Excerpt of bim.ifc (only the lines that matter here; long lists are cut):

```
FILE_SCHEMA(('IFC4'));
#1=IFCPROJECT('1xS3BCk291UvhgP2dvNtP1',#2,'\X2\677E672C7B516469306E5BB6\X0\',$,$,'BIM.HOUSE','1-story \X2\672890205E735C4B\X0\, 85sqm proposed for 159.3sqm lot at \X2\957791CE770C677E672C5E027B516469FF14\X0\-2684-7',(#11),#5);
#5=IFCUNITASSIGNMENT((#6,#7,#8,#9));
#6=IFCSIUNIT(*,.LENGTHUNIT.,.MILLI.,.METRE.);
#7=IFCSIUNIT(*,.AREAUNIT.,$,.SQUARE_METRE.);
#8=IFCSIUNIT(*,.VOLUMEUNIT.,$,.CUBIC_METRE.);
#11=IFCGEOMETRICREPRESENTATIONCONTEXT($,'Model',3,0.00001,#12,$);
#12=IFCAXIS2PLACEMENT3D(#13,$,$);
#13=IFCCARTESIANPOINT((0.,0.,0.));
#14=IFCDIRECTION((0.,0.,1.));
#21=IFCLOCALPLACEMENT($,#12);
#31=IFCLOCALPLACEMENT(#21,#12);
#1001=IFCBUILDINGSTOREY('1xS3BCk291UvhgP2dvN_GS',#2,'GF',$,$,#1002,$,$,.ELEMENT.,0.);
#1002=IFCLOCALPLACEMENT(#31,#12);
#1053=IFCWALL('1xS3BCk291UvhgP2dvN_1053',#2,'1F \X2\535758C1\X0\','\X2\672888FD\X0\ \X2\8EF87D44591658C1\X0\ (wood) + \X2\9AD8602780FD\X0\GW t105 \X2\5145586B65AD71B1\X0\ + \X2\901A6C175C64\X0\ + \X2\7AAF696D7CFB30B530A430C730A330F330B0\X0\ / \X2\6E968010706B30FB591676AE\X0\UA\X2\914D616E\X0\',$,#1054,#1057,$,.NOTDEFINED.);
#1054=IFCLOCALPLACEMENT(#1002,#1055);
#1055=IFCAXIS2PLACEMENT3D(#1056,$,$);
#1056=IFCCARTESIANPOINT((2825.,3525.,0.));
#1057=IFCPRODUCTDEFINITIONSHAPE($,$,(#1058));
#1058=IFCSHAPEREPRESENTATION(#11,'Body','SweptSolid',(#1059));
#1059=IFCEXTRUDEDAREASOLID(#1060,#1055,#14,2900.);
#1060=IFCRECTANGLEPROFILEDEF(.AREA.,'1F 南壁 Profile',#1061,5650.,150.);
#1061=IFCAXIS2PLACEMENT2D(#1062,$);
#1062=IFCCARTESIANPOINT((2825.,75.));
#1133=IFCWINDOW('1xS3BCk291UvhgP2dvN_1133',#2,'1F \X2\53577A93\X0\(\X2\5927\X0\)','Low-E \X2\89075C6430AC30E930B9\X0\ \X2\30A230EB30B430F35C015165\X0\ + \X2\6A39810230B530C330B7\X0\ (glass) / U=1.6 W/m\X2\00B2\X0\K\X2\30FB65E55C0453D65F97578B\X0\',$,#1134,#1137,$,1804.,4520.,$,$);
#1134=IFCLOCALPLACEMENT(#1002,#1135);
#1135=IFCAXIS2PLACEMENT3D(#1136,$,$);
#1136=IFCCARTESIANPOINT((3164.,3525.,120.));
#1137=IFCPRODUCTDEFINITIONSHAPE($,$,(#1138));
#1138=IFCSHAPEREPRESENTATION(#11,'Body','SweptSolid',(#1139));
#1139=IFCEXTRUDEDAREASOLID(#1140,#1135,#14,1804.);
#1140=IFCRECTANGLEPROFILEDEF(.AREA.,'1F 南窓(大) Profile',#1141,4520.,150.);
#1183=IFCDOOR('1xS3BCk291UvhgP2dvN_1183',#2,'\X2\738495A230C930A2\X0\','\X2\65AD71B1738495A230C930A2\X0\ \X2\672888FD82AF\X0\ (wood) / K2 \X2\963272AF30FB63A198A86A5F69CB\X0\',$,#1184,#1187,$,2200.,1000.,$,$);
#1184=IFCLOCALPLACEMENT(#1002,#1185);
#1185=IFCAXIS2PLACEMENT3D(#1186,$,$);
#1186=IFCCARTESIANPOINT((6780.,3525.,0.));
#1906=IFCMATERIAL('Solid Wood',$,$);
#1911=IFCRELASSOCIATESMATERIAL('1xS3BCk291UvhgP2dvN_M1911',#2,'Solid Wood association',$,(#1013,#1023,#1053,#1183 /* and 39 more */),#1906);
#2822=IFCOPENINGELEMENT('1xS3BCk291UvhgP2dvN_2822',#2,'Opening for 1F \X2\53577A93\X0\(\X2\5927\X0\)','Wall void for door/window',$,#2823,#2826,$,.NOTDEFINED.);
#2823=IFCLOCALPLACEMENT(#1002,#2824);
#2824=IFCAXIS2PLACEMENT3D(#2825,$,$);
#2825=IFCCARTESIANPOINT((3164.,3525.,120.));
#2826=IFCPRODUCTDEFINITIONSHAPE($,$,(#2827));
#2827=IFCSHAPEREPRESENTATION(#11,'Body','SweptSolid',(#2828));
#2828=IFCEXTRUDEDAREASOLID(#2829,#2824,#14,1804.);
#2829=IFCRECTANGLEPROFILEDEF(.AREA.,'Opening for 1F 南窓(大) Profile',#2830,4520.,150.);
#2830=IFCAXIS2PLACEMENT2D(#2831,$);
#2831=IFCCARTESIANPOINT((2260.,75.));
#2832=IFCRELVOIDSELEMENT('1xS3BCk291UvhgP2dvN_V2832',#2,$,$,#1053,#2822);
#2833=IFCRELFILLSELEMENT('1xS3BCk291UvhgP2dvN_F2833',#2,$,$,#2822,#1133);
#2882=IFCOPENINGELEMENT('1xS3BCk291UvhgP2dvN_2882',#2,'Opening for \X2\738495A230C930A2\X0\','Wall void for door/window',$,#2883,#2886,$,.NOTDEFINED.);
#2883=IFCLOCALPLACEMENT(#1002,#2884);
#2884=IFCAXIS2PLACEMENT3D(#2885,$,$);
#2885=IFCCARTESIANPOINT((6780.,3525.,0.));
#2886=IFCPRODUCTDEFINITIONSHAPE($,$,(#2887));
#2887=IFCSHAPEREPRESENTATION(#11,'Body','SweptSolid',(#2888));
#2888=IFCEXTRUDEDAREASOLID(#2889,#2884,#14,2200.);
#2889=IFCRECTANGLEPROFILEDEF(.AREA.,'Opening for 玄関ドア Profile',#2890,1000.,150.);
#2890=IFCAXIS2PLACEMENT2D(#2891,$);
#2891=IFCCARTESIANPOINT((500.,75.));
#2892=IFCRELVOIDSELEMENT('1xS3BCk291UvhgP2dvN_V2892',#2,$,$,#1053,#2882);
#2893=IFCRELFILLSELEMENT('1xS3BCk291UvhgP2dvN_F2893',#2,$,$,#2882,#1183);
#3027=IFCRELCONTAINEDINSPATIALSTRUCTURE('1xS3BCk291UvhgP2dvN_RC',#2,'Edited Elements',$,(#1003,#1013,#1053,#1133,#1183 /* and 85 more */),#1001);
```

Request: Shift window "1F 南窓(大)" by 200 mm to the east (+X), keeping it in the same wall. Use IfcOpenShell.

```python
import ifcopenshell
import ifcopenshell.api.geometry
import ifcopenshell.util.placement

model = ifcopenshell.open("bim.ifc")

window = model.by_guid("1xS3BCk291UvhgP2dvN_1133")
opening = window.FillsVoids[0].RelatingOpeningElement
wall = opening.VoidsElements[0].RelatingBuildingElement

wall_matrix = ifcopenshell.util.placement.get_local_placement(wall.ObjectPlacement)
shift = wall_matrix[:3, 0] * 200.0
before = ifcopenshell.util.placement.get_local_placement(window.ObjectPlacement)[:3, 3].copy()

# The window is not placed relative to its opening, so move both.
for product in (opening, window):
    matrix = ifcopenshell.util.placement.get_local_placement(product.ObjectPlacement)
    matrix[:3, 3] += shift
    ifcopenshell.api.geometry.edit_object_placement(model, product=product, matrix=matrix, is_si=False)

after = ifcopenshell.util.placement.get_local_placement(window.ObjectPlacement)[:3, 3]
print("window moved by", (after - before).round(3) + 0.0)

model.write("bim_edited.ifc")
```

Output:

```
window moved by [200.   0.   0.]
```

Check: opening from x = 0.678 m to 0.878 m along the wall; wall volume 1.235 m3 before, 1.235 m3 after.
